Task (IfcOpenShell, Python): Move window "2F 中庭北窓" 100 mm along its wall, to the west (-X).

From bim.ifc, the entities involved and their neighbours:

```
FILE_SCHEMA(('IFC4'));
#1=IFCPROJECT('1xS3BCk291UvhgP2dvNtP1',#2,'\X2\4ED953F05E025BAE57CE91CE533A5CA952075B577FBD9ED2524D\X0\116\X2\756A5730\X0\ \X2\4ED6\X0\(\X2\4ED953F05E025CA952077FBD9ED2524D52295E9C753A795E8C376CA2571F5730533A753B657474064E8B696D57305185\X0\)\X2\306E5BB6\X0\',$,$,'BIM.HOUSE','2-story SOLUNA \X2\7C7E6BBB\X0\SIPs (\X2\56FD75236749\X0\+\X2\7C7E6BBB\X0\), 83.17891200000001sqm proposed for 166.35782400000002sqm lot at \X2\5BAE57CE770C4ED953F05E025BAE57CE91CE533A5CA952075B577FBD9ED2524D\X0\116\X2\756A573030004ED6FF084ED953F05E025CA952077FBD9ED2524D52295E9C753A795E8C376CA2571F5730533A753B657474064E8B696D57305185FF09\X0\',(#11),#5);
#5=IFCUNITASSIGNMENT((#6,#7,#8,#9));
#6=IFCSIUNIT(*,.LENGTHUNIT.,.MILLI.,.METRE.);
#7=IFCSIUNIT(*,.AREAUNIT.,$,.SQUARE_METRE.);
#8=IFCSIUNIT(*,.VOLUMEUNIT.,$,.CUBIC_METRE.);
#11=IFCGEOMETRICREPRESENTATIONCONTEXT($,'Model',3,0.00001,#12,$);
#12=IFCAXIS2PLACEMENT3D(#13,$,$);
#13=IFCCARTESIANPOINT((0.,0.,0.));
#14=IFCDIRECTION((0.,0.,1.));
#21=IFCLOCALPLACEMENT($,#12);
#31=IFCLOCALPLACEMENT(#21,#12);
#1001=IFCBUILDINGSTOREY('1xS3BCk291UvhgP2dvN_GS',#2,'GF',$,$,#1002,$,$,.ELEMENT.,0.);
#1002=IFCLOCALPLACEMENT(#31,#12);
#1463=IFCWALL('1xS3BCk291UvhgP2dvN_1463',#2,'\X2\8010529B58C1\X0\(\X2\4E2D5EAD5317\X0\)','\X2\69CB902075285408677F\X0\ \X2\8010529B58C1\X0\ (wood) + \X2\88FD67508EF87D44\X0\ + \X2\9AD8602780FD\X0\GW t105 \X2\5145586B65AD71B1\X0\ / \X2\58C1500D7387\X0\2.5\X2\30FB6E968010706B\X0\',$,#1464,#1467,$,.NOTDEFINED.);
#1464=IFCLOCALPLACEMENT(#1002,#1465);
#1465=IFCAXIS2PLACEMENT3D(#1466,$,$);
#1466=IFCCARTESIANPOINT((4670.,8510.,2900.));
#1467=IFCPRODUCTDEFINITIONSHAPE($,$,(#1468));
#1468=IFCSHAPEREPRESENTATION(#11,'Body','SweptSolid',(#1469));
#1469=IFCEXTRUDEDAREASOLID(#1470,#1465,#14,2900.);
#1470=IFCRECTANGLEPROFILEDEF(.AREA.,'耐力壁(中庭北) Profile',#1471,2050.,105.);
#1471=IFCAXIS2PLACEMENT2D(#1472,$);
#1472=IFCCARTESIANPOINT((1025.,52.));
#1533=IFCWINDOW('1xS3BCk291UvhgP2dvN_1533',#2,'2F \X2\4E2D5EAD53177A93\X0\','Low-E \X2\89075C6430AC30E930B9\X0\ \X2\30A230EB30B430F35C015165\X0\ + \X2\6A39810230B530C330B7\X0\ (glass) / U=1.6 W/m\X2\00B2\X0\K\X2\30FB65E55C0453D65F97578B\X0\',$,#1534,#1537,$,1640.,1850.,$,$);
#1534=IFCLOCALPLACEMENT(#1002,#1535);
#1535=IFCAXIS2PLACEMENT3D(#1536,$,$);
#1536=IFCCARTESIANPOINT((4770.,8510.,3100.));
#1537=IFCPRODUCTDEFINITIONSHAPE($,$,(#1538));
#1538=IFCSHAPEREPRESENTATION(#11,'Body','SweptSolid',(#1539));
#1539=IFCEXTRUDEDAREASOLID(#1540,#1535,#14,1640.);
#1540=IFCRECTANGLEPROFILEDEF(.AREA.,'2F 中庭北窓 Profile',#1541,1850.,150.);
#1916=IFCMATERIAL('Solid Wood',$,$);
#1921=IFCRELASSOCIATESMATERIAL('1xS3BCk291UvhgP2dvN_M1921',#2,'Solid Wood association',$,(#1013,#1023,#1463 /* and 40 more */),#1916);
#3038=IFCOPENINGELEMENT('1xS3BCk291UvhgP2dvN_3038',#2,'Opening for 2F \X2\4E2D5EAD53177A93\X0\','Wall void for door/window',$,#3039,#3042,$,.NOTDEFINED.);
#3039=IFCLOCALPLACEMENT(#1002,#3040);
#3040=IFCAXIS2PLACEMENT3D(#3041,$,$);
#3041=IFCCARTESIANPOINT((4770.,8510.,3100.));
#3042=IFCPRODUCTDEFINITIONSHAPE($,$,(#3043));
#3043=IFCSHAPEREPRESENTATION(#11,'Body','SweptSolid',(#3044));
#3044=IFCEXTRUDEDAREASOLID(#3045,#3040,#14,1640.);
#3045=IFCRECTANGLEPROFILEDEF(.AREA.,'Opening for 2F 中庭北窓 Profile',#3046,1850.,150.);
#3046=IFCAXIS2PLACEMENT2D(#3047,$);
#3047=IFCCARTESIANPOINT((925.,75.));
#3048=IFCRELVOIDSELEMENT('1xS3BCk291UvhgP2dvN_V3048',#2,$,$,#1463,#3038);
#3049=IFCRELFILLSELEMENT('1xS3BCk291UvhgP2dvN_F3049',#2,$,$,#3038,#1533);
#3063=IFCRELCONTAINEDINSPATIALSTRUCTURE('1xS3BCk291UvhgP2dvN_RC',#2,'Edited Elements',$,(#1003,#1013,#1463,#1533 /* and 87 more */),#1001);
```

```python
import ifcopenshell
import ifcopenshell.api.geometry
import ifcopenshell.util.placement
import ifcopenshell.util.unit

model = ifcopenshell.open("bim.ifc")
unit_scale = ifcopenshell.util.unit.calculate_unit_scale(model)

window = model.by_guid("1xS3BCk291UvhgP2dvN_1533")
opening = window.FillsVoids[0].RelatingOpeningElement
wall = opening.VoidsElements[0].RelatingBuildingElement

wall_matrix = ifcopenshell.util.placement.get_local_placement(wall.ObjectPlacement)
shift = wall_matrix[:3, 0] * -0.1 / unit_scale
before = ifcopenshell.util.placement.get_local_placement(window.ObjectPlacement)[:3, 3].copy()

# The window is not placed relative to its opening, so move both.
for product in (opening, window):
    matrix = ifcopenshell.util.placement.get_local_placement(product.ObjectPlacement)
    matrix[:3, 3] += shift
    ifcopenshell.api.geometry.edit_object_placement(model, product=product, matrix=matrix, is_si=False)

after = ifcopenshell.util.placement.get_local_placement(window.ObjectPlacement)[:3, 3]
print("window moved by", (after - before).round(3) + 0.0)

model.write("bim_updated.ifc")
```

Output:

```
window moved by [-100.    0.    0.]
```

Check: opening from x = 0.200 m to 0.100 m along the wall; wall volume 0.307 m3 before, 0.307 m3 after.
